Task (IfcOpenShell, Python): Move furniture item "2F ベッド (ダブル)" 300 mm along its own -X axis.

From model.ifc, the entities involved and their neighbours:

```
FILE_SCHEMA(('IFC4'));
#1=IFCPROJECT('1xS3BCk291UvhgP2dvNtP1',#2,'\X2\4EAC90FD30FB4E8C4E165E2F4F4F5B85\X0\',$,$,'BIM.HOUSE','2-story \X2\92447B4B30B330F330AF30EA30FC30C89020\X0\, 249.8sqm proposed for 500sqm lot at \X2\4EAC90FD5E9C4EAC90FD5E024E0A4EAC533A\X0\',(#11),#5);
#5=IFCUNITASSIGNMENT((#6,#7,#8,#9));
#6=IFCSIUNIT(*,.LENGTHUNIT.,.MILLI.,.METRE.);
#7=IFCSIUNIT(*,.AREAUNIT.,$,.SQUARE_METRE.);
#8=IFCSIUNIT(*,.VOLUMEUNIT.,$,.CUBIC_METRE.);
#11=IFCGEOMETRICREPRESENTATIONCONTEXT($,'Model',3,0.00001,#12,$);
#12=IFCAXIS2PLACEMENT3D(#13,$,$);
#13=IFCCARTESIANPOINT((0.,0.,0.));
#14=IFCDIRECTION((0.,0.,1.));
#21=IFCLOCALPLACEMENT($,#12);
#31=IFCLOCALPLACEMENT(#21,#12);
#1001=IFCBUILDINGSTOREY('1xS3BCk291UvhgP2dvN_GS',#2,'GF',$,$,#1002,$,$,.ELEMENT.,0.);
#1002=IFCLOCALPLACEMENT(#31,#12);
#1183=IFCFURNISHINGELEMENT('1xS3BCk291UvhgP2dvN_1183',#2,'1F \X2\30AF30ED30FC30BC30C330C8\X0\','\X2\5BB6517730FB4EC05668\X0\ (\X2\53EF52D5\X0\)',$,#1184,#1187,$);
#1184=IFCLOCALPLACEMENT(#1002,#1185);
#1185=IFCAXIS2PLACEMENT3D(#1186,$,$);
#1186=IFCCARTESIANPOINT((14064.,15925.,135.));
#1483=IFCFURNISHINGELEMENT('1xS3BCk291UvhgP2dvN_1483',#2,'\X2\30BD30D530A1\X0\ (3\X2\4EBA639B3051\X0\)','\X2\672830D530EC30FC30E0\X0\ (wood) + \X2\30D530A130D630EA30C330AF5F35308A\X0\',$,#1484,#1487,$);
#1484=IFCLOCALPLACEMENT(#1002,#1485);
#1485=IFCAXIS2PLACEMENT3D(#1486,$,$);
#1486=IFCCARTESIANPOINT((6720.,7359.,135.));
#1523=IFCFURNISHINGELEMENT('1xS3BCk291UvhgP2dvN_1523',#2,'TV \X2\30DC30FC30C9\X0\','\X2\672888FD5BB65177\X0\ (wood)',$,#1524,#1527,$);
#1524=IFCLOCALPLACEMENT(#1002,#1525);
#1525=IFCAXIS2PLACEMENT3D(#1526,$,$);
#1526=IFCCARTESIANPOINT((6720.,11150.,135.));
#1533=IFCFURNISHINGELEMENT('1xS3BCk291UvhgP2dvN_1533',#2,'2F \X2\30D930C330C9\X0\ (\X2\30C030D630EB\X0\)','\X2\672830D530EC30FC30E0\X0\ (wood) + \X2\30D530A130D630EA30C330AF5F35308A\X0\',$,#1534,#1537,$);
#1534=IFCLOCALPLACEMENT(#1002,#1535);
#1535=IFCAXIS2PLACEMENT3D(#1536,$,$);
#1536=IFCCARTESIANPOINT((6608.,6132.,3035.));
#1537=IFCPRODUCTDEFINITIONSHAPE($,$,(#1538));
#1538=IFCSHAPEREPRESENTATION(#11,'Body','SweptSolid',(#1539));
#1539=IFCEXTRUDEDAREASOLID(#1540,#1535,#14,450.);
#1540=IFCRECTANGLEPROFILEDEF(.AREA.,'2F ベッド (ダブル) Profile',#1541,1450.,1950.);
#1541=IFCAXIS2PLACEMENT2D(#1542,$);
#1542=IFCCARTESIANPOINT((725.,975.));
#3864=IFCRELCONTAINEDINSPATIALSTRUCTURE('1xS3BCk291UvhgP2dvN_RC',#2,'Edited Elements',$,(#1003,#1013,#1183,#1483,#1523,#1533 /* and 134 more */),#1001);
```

```python
import ifcopenshell
import ifcopenshell.api.geometry
import ifcopenshell.util.placement
import ifcopenshell.util.unit

model = ifcopenshell.open("model.ifc")
unit_scale = ifcopenshell.util.unit.calculate_unit_scale(model)

item = model.by_guid("1xS3BCk291UvhgP2dvN_1533")
matrix = ifcopenshell.util.placement.get_local_placement(item.ObjectPlacement)
matrix[:3, 3] -= matrix[:3, 0] * 0.3 / unit_scale
ifcopenshell.api.geometry.edit_object_placement(model, product=item, matrix=matrix, is_si=False)

print(ifcopenshell.util.placement.get_local_placement(item.ObjectPlacement).round(3) + 0.0)

model.write("model_updated.ifc")
```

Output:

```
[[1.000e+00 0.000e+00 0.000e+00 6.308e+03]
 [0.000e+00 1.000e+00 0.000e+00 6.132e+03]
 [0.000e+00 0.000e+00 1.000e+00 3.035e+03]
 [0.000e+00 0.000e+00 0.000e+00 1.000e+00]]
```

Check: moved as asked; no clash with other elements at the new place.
